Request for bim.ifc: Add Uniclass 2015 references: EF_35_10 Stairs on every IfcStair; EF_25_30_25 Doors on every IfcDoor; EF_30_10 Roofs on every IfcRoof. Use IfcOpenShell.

First a look at what the model holds.

```python
import ifcopenshell

model = ifcopenshell.open("bim.ifc")
print(model.schema)
print("classifications:", [c.Name for c in model.by_type("IfcClassification")])
for ifc_class in ("IfcDoor", "IfcRoof", "IfcStair", "IfcWall", "IfcWindow"):
    print(ifc_class, len(model.by_type(ifc_class)))
```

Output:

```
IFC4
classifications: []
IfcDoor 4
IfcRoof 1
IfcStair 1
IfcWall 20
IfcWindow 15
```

```python
import ifcopenshell
import ifcopenshell.api.classification

model = ifcopenshell.open("bim.ifc")

system = ifcopenshell.api.classification.add_classification(model, classification="Uniclass 2015")

codes = {
    "IfcStair": ("EF_35_10", "Stairs"),
    "IfcDoor": ("EF_25_30_25", "Doors"),
    "IfcRoof": ("EF_30_10", "Roofs"),
}
for ifc_class, (code, name) in codes.items():
    products = model.by_type(ifc_class)
    ifcopenshell.api.classification.add_reference(
        model, products=products, classification=system, identification=code, name=name
    )
    print(code, len(products))

model.write("bim_updated.ifc")
```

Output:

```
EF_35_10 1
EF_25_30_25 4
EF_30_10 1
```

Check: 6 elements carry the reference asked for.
